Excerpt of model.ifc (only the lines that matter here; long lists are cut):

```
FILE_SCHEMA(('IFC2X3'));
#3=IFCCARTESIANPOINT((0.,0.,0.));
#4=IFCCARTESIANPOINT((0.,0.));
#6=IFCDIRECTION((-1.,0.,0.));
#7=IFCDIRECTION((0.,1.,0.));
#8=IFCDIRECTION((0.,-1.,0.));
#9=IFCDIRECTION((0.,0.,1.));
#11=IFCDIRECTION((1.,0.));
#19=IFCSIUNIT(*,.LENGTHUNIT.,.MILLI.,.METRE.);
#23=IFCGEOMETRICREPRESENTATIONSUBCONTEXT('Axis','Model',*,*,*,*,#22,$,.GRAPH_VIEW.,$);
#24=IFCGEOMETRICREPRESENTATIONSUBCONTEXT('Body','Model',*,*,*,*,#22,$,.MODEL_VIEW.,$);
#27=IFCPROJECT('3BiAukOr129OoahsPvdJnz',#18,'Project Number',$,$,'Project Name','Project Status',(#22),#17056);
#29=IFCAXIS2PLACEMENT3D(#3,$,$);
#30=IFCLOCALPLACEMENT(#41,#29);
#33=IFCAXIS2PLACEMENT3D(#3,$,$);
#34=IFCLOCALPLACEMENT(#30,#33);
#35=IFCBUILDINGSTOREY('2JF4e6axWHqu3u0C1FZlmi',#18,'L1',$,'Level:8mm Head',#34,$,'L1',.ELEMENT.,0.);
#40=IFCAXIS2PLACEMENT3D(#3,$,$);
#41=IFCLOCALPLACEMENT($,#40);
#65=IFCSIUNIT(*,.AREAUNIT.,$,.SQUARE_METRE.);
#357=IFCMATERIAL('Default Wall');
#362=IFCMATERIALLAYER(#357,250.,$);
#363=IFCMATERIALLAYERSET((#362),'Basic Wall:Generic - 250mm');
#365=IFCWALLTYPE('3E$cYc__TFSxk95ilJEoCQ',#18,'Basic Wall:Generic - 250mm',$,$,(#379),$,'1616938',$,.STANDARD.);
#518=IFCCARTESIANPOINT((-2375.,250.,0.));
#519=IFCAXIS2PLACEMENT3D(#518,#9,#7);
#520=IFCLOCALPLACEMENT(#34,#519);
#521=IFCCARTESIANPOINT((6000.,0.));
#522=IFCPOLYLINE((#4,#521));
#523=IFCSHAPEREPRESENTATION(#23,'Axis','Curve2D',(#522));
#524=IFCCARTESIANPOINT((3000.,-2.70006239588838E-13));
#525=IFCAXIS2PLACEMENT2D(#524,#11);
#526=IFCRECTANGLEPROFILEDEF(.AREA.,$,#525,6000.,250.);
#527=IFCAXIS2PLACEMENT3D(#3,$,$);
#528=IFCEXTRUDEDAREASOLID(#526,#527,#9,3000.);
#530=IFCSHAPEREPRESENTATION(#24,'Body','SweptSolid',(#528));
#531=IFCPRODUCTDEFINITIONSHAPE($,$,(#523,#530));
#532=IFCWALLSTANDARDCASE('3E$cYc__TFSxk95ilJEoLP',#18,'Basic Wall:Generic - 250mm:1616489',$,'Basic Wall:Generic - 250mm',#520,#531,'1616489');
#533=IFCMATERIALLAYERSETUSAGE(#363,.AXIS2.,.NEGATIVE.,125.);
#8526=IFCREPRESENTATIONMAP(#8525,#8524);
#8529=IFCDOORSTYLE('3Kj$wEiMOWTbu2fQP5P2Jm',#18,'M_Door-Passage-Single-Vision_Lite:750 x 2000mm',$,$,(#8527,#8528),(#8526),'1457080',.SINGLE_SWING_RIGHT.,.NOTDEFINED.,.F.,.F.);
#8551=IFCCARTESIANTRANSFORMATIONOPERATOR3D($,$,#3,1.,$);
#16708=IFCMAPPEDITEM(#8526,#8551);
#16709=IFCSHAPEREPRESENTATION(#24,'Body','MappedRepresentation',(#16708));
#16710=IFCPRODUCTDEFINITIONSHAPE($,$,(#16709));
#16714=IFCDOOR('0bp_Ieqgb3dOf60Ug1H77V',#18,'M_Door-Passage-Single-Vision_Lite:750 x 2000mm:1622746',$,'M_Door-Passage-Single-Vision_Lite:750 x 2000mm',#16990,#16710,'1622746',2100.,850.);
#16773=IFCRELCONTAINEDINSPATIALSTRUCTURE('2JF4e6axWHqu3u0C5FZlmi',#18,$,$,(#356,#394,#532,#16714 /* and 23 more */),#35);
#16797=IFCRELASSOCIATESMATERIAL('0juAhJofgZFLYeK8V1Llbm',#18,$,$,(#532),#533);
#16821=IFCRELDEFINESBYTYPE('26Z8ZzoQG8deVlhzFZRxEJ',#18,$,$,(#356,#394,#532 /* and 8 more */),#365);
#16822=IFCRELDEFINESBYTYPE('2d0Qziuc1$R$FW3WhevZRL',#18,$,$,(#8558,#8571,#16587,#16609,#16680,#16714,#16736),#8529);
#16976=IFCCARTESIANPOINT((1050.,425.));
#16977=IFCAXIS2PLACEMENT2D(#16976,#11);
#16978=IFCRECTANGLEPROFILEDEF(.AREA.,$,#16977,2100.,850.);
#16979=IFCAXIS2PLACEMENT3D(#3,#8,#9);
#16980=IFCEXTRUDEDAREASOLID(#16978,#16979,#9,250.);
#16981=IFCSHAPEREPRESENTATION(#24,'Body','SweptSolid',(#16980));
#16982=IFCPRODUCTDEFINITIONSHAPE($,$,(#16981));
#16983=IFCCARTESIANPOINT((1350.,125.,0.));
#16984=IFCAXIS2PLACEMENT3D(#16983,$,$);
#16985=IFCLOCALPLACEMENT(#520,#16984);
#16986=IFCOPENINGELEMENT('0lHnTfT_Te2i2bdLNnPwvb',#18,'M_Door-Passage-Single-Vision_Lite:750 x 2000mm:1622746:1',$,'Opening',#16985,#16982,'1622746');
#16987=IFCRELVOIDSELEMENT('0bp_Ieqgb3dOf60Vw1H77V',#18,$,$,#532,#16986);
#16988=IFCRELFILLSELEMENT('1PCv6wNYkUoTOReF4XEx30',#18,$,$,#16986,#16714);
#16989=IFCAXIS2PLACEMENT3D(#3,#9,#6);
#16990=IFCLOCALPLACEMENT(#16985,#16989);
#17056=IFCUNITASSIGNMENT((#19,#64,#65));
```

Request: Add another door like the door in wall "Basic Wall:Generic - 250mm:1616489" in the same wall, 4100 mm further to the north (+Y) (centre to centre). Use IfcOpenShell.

```python
import ifcopenshell
import ifcopenshell.api.feature
import ifcopenshell.api.geometry
import ifcopenshell.api.root
import ifcopenshell.geom
import ifcopenshell.util.element
import ifcopenshell.util.placement
import ifcopenshell.util.shape
import ifcopenshell.util.unit

model = ifcopenshell.open("model.ifc")
unit_scale = ifcopenshell.util.unit.calculate_unit_scale(model)
settings = ifcopenshell.geom.settings()


def volume(element):
    """Net volume in cubic metres, openings subtracted."""
    shape = ifcopenshell.geom.create_shape(settings, element)
    return ifcopenshell.util.shape.get_volume(shape.geometry)


def reuse_history(source, copy):
    """copy_class also copies each property set's owner history, people and application; keep the originals."""
    for rel in copy.IsDefinedBy:
        if rel.is_a("IfcRelDefinesByProperties") and (history := rel.RelatingPropertyDefinition.OwnerHistory):
            rel.RelatingPropertyDefinition.OwnerHistory = source.OwnerHistory
            ifcopenshell.util.element.remove_deep2(model, history)


door = model.by_id(16714)
opening = door.FillsVoids[0].RelatingOpeningElement
wall = opening.VoidsElements[0].RelatingBuildingElement
before = volume(wall)
shift = ifcopenshell.util.placement.get_local_placement(wall.ObjectPlacement)[:3, 0] * 4.1 / unit_scale

# copy_class copies the void relationship, type, container and properties, but no geometry.
new_opening = ifcopenshell.api.root.copy_class(model, product=opening)
new_opening.Representation = ifcopenshell.util.element.copy_deep(
    model, opening.Representation, exclude=["IfcGeometricRepresentationContext", "IfcRepresentationMap"]
)
new_opening.Name = "M_Door-Passage-Single-Vision_Lite:750 x 2000mm"
new_opening.Tag = None
new_door = ifcopenshell.api.root.copy_class(model, product=door)
new_door.Representation = ifcopenshell.util.element.copy_deep(
    model, door.Representation, exclude=["IfcGeometricRepresentationContext", "IfcRepresentationMap"]
)
new_door.Name = "M_Door-Passage-Single-Vision_Lite:750 x 2000mm"
new_door.Tag = None
reuse_history(door, new_door)
fills = ifcopenshell.api.feature.add_filling(model, opening=new_opening, element=new_door)
fills.OwnerHistory = new_door.OwnerHistory  # required in IFC2X3

for old, new in ((opening, new_opening), (door, new_door)):
    matrix = ifcopenshell.util.placement.get_local_placement(old.ObjectPlacement)
    matrix[:3, 3] += shift
    ifcopenshell.api.geometry.edit_object_placement(model, product=new, matrix=matrix, is_si=False)

after = volume(wall)

print(f"wall volume {before:.3f} -> {after:.3f} m3")

model.write("model_edited.ifc")
```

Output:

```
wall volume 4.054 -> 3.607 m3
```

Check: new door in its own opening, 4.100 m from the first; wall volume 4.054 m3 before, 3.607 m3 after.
